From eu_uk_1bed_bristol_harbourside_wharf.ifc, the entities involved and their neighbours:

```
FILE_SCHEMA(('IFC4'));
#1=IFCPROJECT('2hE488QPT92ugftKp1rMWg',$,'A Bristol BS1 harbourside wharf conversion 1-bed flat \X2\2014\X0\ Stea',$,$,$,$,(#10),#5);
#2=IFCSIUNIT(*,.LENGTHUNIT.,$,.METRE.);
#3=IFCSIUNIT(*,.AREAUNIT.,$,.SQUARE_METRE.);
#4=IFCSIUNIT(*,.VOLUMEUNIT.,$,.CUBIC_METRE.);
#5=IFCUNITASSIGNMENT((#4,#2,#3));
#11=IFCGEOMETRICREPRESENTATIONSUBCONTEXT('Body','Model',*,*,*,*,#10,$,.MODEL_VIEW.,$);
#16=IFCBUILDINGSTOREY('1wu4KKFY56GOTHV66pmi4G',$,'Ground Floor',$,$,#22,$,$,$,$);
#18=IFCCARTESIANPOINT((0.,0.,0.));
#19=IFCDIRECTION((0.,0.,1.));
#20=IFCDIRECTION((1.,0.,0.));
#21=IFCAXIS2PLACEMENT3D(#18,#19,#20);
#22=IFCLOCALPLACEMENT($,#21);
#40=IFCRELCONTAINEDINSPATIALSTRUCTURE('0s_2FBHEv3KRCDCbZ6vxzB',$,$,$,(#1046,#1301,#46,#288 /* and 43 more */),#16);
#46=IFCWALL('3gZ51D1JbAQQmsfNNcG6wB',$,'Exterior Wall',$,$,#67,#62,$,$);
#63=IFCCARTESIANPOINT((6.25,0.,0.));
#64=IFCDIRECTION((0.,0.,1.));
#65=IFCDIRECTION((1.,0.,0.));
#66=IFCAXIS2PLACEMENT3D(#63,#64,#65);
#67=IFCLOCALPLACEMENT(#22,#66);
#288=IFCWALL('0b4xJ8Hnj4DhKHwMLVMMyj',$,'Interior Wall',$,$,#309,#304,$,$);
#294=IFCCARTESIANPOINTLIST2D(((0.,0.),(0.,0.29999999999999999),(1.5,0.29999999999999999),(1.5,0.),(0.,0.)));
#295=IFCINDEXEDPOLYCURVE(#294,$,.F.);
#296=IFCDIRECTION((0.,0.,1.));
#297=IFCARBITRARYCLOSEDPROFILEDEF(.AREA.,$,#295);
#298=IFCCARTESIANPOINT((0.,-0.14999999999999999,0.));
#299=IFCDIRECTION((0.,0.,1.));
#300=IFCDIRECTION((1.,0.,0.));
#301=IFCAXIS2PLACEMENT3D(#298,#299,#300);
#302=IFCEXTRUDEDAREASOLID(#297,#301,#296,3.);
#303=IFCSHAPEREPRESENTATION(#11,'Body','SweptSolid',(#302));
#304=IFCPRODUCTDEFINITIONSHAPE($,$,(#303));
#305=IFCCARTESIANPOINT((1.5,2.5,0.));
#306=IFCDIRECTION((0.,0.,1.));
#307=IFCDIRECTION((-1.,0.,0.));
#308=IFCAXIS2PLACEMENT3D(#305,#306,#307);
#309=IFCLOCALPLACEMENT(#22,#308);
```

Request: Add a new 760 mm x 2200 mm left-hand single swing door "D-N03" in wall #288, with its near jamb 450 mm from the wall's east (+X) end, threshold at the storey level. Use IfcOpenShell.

```python
import numpy as np
import ifcopenshell
import ifcopenshell.api.feature
import ifcopenshell.api.geometry
import ifcopenshell.api.root
import ifcopenshell.api.spatial
import ifcopenshell.geom
import ifcopenshell.util.element
import ifcopenshell.util.placement
import ifcopenshell.util.representation
import ifcopenshell.util.shape
import ifcopenshell.util.unit

model = ifcopenshell.open("eu_uk_1bed_bristol_harbourside_wharf.ifc")
unit_scale = ifcopenshell.util.unit.calculate_unit_scale(model)
settings = ifcopenshell.geom.settings()


def volume(element):
    """Net volume in cubic metres, openings subtracted."""
    shape = ifcopenshell.geom.create_shape(settings, element)
    return ifcopenshell.util.shape.get_volume(shape.geometry)


wall = model.by_guid("0b4xJ8Hnj4DhKHwMLVMMyj")
storey = ifcopenshell.util.element.get_container(wall, ifc_class="IfcBuildingStorey")
context = ifcopenshell.util.representation.get_context(model, "Model", "Body", "MODEL_VIEW")
before = volume(wall)

width, height, from_end, sill = 0.76, 2.2, 0.45, 0.0  # metres

# The wall runs along its own X axis, and the end named is its -X end.
wall_shape = ifcopenshell.geom.create_shape(settings, wall)
x, y, z = ifcopenshell.util.shape.get_vertices(wall_shape.geometry).T
start = x.min() + from_end
face, thickness = float(y.min()), float(y.max() - y.min())
wall_matrix = ifcopenshell.util.placement.get_local_placement(wall.ObjectPlacement)
level = ifcopenshell.util.placement.get_local_placement(storey.ObjectPlacement)[2, 3]


def in_wall(x, y):
    """Placement at x, y metres in the wall's axes, at sill height."""
    matrix = wall_matrix.copy()
    matrix[:, 3] = wall_matrix @ np.array([x / unit_scale, y / unit_scale, 0.0, 1.0])
    matrix[2, 3] = level + sill / unit_scale
    return matrix


# Opening: a box that overshoots both wall faces by 50 mm.
opening = ifcopenshell.api.root.create_entity(model, ifc_class="IfcOpeningElement", predefined_type="OPENING")
box = ifcopenshell.api.geometry.add_wall_representation(
    model, context=context, length=width, height=height, thickness=thickness + 0.1
)
ifcopenshell.api.geometry.assign_representation(model, product=opening, representation=box)
ifcopenshell.api.geometry.edit_object_placement(model, product=opening, matrix=in_wall(start, face - 0.05), is_si=False)
ifcopenshell.api.feature.add_feature(model, feature=opening, element=wall)

door = ifcopenshell.api.root.create_entity(model, ifc_class="IfcDoor", name="D-N03", predefined_type="DOOR")
door.OverallWidth, door.OverallHeight = width / unit_scale, height / unit_scale
door.OperationType = "SINGLE_SWING_LEFT"
body = ifcopenshell.api.geometry.add_door_representation(
    model,
    context=context,
    overall_width=door.OverallWidth,
    overall_height=door.OverallHeight,
    operation_type="SINGLE_SWING_LEFT",
    lining_properties={"LiningDepth": thickness / unit_scale, "ThresholdDepth": thickness / unit_scale},
)
ifcopenshell.api.geometry.assign_representation(model, product=door, representation=body)
ifcopenshell.api.spatial.assign_container(model, products=[door], relating_structure=storey)
ifcopenshell.api.feature.add_filling(model, opening=opening, element=door)

# The lining spans the wall, so the door starts at the wall face.
ifcopenshell.api.geometry.edit_object_placement(model, product=door, matrix=in_wall(start, face), is_si=False)

after = volume(wall)

print(f"wall volume {before:.3f} -> {after:.3f} m3")

model.write("eu_uk_1bed_bristol_harbourside_wharf_rev.ifc")
```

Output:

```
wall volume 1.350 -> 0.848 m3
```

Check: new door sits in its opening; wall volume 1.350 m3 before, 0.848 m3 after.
